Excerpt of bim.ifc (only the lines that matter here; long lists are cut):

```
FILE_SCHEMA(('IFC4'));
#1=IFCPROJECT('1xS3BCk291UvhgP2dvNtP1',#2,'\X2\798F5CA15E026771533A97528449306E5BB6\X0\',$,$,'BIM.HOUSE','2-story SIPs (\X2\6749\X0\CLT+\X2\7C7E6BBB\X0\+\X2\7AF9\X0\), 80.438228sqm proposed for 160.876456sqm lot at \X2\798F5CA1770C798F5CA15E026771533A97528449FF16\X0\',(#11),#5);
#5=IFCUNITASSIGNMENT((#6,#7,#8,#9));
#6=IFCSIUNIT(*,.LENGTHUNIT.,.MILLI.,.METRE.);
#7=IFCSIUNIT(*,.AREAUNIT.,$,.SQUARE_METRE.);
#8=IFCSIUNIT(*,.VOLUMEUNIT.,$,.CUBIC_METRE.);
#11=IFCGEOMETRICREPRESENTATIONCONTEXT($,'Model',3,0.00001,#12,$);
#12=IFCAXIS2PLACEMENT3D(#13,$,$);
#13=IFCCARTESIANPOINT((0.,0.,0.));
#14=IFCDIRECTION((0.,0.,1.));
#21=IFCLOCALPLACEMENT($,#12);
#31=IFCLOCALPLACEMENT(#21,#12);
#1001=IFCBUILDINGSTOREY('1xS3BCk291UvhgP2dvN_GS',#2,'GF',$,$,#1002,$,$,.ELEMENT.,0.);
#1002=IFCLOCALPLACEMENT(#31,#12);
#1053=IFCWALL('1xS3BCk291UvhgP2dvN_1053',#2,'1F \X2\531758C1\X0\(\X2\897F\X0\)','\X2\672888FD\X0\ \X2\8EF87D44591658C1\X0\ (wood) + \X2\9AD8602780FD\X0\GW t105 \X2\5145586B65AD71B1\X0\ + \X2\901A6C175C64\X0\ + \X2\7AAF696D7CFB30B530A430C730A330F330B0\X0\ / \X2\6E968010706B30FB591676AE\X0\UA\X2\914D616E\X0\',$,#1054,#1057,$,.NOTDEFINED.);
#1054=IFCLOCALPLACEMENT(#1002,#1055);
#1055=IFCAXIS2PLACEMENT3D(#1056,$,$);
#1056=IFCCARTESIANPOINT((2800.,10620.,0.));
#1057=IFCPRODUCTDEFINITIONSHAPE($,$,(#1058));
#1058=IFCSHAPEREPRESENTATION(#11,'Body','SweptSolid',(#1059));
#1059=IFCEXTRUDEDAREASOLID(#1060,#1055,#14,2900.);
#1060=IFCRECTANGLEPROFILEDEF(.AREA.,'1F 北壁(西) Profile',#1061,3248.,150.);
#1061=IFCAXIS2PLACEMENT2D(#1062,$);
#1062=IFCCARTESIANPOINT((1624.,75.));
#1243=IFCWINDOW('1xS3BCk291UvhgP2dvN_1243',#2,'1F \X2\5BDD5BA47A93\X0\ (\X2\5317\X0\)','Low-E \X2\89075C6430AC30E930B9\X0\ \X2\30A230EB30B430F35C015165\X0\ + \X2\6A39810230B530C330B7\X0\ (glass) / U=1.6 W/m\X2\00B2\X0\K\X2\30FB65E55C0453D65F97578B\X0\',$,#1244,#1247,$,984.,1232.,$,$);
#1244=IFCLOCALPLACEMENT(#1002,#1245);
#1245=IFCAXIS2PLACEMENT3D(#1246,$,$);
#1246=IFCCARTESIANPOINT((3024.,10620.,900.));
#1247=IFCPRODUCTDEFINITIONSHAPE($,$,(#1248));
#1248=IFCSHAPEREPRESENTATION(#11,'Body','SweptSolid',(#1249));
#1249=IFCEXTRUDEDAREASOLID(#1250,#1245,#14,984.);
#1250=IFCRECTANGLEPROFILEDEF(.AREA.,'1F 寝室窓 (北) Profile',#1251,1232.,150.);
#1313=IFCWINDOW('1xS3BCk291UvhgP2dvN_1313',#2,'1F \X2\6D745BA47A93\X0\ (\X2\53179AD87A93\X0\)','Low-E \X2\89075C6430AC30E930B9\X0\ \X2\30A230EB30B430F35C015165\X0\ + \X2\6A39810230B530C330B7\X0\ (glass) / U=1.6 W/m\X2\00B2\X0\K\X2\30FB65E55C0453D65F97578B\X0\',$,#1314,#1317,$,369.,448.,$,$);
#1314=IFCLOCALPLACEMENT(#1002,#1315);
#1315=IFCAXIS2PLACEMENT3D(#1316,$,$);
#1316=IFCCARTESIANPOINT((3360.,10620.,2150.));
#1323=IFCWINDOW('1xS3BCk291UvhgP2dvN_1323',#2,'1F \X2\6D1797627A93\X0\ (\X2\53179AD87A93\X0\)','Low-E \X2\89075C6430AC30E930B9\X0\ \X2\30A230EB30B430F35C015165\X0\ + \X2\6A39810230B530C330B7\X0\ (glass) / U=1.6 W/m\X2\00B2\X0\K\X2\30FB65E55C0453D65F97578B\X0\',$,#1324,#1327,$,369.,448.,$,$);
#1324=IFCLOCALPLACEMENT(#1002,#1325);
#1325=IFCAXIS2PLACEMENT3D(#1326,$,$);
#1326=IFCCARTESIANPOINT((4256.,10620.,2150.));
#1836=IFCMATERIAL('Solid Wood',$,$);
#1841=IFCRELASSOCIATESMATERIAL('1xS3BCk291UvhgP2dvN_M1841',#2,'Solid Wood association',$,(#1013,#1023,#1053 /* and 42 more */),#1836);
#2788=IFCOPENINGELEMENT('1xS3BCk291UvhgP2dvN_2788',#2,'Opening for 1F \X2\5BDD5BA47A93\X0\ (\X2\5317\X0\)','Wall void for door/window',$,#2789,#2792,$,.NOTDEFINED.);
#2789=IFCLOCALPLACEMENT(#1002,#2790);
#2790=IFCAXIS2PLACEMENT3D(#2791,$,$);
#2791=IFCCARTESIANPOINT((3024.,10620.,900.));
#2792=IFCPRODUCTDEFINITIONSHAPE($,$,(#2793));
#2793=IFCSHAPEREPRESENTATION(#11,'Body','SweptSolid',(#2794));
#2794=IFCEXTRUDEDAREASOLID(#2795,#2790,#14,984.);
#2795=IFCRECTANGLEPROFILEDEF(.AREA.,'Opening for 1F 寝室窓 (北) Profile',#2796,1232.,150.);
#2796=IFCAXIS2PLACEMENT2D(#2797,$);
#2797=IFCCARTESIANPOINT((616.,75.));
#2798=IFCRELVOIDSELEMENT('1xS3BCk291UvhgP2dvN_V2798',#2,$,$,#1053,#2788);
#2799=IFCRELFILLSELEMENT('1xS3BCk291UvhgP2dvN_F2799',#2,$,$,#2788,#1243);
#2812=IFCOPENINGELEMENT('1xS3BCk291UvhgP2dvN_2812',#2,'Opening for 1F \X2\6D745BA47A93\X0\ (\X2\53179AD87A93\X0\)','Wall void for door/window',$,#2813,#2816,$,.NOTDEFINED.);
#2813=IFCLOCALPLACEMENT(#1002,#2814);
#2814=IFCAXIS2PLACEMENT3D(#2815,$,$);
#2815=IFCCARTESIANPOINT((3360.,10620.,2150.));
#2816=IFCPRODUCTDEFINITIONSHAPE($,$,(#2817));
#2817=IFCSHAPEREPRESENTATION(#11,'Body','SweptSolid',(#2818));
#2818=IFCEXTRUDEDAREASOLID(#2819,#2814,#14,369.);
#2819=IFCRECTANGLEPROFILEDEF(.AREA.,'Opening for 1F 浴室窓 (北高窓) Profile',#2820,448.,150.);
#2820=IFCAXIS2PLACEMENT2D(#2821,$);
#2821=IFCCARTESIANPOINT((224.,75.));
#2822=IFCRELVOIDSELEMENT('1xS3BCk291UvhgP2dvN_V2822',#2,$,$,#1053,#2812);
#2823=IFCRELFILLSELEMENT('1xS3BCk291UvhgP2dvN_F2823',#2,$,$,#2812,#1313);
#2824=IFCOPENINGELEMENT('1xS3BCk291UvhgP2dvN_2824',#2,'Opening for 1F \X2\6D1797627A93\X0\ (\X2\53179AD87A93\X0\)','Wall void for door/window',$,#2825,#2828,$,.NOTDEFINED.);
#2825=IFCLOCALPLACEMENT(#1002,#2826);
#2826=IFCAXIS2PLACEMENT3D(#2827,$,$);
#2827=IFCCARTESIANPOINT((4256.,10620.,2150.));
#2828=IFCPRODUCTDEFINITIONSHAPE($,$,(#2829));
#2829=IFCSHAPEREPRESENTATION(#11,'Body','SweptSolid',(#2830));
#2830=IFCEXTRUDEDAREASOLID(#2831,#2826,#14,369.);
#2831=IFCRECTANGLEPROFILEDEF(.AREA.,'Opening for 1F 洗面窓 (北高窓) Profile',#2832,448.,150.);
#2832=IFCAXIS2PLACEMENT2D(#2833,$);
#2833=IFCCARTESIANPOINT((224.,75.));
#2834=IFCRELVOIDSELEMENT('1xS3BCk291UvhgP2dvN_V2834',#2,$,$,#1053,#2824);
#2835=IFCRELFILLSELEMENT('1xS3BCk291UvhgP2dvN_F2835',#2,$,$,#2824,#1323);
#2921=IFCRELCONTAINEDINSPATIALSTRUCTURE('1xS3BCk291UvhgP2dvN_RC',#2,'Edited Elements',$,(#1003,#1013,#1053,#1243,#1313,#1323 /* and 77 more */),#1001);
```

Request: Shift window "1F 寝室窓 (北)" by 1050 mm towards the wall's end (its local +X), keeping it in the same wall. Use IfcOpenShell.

```python
import ifcopenshell
import ifcopenshell.api.geometry
import ifcopenshell.util.placement

model = ifcopenshell.open("bim.ifc")

window = model.by_id(1243)
opening = window.FillsVoids[0].RelatingOpeningElement
wall = opening.VoidsElements[0].RelatingBuildingElement

wall_matrix = ifcopenshell.util.placement.get_local_placement(wall.ObjectPlacement)
shift = wall_matrix[:3, 0] * 1050.0
before = ifcopenshell.util.placement.get_local_placement(window.ObjectPlacement)[:3, 3].copy()

# The window is not placed relative to its opening, so move both.
for product in (opening, window):
    matrix = ifcopenshell.util.placement.get_local_placement(product.ObjectPlacement)
    matrix[:3, 3] += shift
    ifcopenshell.api.geometry.edit_object_placement(model, product=product, matrix=matrix, is_si=False)

after = ifcopenshell.util.placement.get_local_placement(window.ObjectPlacement)[:3, 3]
print("window moved by", (after - before).round(3) + 0.0)

model.write("bim-out.ifc")
```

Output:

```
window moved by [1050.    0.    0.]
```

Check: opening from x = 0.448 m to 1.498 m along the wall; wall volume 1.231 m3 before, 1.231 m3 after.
